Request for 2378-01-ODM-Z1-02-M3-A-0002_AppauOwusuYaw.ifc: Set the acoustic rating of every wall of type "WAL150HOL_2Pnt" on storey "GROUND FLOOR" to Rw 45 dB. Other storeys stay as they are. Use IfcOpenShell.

First a look at what the model holds.

```python
import ifcopenshell
import ifcopenshell.util.element

model = ifcopenshell.open("2378-01-ODM-Z1-02-M3-A-0002_AppauOwusuYaw.ifc")
print(model.schema)
storey = next(s for s in model.by_type("IfcBuildingStorey") if s.Name == "GROUND FLOOR")
walls = [e for e in ifcopenshell.util.element.get_decomposition(storey) if e.is_a("IfcWall")]
seen = {}
for e in walls:
    element_type = ifcopenshell.util.element.get_type(e)
    key = (element_type.Name if element_type != e and element_type else None, ifcopenshell.util.element.get_pset(e, "Pset_WallCommon", "AcousticRating"))
    seen[key] = seen.get(key, 0) + 1
for (name, value), count in sorted(seen.items(), key=str):
    print(count, "x", name, "|", value)
```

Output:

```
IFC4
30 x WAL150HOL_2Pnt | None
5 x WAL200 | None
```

```python
import ifcopenshell
import ifcopenshell.api.pset
import ifcopenshell.util.element

model = ifcopenshell.open("2378-01-ODM-Z1-02-M3-A-0002_AppauOwusuYaw.ifc")

storey = next(s for s in model.by_type("IfcBuildingStorey") if s.Name == "GROUND FLOOR")
walls = [e for e in ifcopenshell.util.element.get_decomposition(storey) if e.is_a("IfcWall")]

count = 0
for e in walls:
    element_type = ifcopenshell.util.element.get_type(e)
    if element_type in (None, e) or element_type.Name != "WAL150HOL_2Pnt":
        continue
    # add_pset returns the element's existing set when there is one.
    pset = ifcopenshell.api.pset.add_pset(model, product=e, name="Pset_WallCommon")
    ifcopenshell.api.pset.edit_pset(model, pset=pset, properties={"AcousticRating": "Rw 45 dB"})
    count += 1

print(count, "walls updated")

model.write("2378-01-ODM-Z1-02-M3-A-0002_AppauOwusuYaw_edited.ifc")
```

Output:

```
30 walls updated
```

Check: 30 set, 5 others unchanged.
